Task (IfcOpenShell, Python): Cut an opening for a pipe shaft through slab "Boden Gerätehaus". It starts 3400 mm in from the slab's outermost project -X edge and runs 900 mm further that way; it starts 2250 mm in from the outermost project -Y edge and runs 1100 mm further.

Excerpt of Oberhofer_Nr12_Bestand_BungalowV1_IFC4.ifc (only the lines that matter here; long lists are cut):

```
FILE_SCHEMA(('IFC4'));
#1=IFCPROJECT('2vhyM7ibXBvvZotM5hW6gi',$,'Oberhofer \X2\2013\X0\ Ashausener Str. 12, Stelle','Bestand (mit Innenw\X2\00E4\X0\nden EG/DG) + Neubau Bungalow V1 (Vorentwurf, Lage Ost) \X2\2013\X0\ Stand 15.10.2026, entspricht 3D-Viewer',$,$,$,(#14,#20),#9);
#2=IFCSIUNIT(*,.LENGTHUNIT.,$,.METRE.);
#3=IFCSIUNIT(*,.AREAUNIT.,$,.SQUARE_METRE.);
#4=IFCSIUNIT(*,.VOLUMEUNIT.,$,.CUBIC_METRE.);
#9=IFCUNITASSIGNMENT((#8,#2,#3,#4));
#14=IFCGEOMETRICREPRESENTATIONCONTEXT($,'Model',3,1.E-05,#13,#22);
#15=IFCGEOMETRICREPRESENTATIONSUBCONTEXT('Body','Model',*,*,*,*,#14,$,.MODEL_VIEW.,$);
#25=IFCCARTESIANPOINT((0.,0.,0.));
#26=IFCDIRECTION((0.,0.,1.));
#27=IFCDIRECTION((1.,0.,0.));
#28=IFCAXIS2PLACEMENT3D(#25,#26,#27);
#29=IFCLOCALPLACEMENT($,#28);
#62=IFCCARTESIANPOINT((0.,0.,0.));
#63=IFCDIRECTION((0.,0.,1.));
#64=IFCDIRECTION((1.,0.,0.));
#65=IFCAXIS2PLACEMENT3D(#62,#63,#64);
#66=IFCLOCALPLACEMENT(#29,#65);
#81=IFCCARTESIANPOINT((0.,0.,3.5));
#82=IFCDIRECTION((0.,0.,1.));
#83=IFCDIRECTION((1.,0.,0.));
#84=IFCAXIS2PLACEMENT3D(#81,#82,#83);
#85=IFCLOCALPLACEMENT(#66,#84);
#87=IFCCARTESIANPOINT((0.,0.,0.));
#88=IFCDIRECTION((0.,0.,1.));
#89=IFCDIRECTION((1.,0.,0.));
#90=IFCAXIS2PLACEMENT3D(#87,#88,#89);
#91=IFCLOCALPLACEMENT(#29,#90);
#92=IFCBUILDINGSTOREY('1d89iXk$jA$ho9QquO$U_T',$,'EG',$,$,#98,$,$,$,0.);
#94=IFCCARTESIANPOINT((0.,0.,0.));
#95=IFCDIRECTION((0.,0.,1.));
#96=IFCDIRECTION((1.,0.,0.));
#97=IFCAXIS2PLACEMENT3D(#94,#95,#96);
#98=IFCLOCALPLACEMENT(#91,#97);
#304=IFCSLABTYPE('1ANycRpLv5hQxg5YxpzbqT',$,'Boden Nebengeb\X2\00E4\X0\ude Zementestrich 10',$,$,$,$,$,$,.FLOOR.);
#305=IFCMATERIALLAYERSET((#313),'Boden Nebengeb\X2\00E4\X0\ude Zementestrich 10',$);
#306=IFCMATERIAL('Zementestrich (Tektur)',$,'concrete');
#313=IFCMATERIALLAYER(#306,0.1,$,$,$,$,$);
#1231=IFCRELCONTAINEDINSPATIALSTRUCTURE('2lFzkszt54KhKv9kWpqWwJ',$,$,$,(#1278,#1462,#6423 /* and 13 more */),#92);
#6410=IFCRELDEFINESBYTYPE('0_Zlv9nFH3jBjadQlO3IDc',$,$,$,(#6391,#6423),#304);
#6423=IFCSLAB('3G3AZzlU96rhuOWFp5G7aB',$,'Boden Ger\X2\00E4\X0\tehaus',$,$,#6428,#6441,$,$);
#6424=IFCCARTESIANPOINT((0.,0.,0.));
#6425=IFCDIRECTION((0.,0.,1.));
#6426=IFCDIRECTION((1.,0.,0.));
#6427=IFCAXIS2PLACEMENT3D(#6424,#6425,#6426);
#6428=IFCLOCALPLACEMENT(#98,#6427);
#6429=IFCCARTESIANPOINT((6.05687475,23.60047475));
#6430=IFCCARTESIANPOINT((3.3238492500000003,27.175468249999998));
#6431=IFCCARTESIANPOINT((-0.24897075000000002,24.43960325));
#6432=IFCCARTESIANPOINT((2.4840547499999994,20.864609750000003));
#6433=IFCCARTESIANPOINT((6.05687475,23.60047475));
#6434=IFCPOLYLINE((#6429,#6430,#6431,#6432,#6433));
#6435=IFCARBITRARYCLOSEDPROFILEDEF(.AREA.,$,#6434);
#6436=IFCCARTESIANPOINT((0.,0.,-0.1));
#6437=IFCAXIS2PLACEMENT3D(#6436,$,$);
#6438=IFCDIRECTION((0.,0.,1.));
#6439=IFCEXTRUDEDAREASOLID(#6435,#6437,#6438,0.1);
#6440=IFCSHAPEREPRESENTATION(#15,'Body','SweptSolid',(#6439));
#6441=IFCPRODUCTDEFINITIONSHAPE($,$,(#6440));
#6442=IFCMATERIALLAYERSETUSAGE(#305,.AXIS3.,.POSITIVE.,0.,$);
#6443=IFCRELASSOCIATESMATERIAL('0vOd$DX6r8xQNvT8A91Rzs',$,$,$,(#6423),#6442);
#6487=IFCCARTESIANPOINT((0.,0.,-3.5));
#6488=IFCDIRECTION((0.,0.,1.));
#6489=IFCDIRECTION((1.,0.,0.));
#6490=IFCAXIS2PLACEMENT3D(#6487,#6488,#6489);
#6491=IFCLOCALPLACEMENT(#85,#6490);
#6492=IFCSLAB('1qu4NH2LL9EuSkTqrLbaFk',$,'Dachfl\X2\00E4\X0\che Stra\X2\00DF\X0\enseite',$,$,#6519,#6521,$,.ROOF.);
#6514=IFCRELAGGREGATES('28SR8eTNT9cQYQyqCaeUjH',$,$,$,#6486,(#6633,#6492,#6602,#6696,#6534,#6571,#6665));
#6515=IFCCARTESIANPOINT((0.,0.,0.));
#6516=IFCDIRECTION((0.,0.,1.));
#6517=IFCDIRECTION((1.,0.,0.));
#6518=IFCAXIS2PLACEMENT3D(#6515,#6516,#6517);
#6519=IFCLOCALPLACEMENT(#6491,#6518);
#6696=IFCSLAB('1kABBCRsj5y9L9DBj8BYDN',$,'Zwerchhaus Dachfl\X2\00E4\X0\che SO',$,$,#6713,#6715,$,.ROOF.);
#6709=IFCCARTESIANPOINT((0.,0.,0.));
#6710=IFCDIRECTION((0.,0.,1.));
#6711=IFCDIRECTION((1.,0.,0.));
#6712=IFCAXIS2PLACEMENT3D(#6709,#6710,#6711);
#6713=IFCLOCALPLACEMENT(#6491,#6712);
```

```python
import numpy as np
import ifcopenshell
import ifcopenshell.api.feature
import ifcopenshell.api.geometry
import ifcopenshell.api.root
import ifcopenshell.geom
import ifcopenshell.util.placement
import ifcopenshell.util.representation
import ifcopenshell.util.shape
import ifcopenshell.util.unit

model = ifcopenshell.open("Oberhofer_Nr12_Bestand_BungalowV1_IFC4.ifc")
unit_scale = ifcopenshell.util.unit.calculate_unit_scale(model)
settings = ifcopenshell.geom.settings()


def volume(element):
    """Net volume in cubic metres, openings subtracted."""
    shape = ifcopenshell.geom.create_shape(settings, element)
    return ifcopenshell.util.shape.get_volume(shape.geometry)


slab = model.by_guid("3G3AZzlU96rhuOWFp5G7aB")
before = volume(slab)

# Extent in the slab's own axes, in metres. The edges named are its -X and -Y sides.
slab_shape = ifcopenshell.geom.create_shape(settings, slab)
vertices = ifcopenshell.util.shape.get_vertices(slab_shape.geometry)
x_min, y_min, bottom = vertices.min(axis=0)
top = vertices[:, 2].max()

opening = ifcopenshell.api.root.create_entity(model, ifc_class="IfcOpeningElement", name="Pipe shaft opening", predefined_type="OPENING")
context = ifcopenshell.util.representation.get_context(model, "Model", "Body", "MODEL_VIEW")
width, depth = 0.9, 1.1
outline = [(0.0, 0.0), (width, 0.0), (width, depth), (0.0, depth), (0.0, 0.0)]
# Overshoot both faces by 50 mm so the cut is clean.
shape = ifcopenshell.api.geometry.add_slab_representation(
    model, context=context, depth=top - bottom + 0.1, polyline=outline
)
ifcopenshell.api.geometry.assign_representation(model, product=opening, representation=shape)

matrix = ifcopenshell.util.placement.get_local_placement(slab.ObjectPlacement)
matrix[:, 3] = matrix @ np.append(np.array([x_min + 3.4, y_min + 2.25, bottom - 0.05]) / unit_scale, 1.0)
ifcopenshell.api.geometry.edit_object_placement(model, product=opening, matrix=matrix, is_si=False)
ifcopenshell.api.feature.add_feature(model, feature=opening, element=slab)

after = volume(slab)

print(f"slab volume {before:.3f} -> {after:.3f} m3")

model.write("Oberhofer_Nr12_Bestand_BungalowV1_IFC4_updated.ifc")
```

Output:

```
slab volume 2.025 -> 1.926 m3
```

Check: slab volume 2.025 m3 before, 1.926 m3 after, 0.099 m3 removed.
